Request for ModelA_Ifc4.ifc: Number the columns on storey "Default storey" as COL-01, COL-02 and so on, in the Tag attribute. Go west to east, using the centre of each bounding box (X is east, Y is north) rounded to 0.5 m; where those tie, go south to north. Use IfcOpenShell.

First a look at what the model holds.

```python
import ifcopenshell
import ifcopenshell.util.element
import ifcopenshell.util.placement

model = ifcopenshell.open("ModelA_Ifc4.ifc")
print(model.schema)
storey = next(s for s in model.by_type("IfcBuildingStorey") if s.Name == "Default storey")
columns = [e for e in ifcopenshell.util.element.get_decomposition(storey) if e.is_a("IfcColumn")]
for e in sorted(columns, key=lambda e: e.id()):
    origin = ifcopenshell.util.placement.get_local_placement(e.ObjectPlacement)[:3, 3]
    print(e.id(), e.Tag, e.Name, origin.round(2) + 0.0, sep=" | ")
```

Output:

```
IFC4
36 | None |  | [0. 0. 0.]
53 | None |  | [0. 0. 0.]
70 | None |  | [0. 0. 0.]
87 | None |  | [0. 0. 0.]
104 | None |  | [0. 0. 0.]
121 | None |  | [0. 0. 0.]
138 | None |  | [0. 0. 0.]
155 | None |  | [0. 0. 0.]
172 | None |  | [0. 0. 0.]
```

```python
import ifcopenshell
import ifcopenshell.geom
import ifcopenshell.util.element
import ifcopenshell.util.shape

model = ifcopenshell.open("ModelA_Ifc4.ifc")
settings = ifcopenshell.geom.settings()
settings.set("use-world-coords", True)


def centre(element):
    shape = ifcopenshell.geom.create_shape(settings, element)
    return ifcopenshell.util.shape.get_bbox_centroid(shape.geometry)


storey = next(s for s in model.by_type("IfcBuildingStorey") if s.Name == "Default storey")
columns = [e for e in ifcopenshell.util.element.get_decomposition(storey) if e.is_a("IfcColumn")]

# Insertion points can sit at a corner or the storey origin, so sort by the geometry (in metres).
centres = {e: centre(e) for e in columns}
columns.sort(key=lambda e: (round(centres[e][0] / 0.5), centres[e][1]))

for i, e in enumerate(columns, start=1):
    number = f"COL-{i:02d}"
    e.Tag = number
    print(e.id(), number)

model.write("ModelA_Ifc4-out.ifc")
```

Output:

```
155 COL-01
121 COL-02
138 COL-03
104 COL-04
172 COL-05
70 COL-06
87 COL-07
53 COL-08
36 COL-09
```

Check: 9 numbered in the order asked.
